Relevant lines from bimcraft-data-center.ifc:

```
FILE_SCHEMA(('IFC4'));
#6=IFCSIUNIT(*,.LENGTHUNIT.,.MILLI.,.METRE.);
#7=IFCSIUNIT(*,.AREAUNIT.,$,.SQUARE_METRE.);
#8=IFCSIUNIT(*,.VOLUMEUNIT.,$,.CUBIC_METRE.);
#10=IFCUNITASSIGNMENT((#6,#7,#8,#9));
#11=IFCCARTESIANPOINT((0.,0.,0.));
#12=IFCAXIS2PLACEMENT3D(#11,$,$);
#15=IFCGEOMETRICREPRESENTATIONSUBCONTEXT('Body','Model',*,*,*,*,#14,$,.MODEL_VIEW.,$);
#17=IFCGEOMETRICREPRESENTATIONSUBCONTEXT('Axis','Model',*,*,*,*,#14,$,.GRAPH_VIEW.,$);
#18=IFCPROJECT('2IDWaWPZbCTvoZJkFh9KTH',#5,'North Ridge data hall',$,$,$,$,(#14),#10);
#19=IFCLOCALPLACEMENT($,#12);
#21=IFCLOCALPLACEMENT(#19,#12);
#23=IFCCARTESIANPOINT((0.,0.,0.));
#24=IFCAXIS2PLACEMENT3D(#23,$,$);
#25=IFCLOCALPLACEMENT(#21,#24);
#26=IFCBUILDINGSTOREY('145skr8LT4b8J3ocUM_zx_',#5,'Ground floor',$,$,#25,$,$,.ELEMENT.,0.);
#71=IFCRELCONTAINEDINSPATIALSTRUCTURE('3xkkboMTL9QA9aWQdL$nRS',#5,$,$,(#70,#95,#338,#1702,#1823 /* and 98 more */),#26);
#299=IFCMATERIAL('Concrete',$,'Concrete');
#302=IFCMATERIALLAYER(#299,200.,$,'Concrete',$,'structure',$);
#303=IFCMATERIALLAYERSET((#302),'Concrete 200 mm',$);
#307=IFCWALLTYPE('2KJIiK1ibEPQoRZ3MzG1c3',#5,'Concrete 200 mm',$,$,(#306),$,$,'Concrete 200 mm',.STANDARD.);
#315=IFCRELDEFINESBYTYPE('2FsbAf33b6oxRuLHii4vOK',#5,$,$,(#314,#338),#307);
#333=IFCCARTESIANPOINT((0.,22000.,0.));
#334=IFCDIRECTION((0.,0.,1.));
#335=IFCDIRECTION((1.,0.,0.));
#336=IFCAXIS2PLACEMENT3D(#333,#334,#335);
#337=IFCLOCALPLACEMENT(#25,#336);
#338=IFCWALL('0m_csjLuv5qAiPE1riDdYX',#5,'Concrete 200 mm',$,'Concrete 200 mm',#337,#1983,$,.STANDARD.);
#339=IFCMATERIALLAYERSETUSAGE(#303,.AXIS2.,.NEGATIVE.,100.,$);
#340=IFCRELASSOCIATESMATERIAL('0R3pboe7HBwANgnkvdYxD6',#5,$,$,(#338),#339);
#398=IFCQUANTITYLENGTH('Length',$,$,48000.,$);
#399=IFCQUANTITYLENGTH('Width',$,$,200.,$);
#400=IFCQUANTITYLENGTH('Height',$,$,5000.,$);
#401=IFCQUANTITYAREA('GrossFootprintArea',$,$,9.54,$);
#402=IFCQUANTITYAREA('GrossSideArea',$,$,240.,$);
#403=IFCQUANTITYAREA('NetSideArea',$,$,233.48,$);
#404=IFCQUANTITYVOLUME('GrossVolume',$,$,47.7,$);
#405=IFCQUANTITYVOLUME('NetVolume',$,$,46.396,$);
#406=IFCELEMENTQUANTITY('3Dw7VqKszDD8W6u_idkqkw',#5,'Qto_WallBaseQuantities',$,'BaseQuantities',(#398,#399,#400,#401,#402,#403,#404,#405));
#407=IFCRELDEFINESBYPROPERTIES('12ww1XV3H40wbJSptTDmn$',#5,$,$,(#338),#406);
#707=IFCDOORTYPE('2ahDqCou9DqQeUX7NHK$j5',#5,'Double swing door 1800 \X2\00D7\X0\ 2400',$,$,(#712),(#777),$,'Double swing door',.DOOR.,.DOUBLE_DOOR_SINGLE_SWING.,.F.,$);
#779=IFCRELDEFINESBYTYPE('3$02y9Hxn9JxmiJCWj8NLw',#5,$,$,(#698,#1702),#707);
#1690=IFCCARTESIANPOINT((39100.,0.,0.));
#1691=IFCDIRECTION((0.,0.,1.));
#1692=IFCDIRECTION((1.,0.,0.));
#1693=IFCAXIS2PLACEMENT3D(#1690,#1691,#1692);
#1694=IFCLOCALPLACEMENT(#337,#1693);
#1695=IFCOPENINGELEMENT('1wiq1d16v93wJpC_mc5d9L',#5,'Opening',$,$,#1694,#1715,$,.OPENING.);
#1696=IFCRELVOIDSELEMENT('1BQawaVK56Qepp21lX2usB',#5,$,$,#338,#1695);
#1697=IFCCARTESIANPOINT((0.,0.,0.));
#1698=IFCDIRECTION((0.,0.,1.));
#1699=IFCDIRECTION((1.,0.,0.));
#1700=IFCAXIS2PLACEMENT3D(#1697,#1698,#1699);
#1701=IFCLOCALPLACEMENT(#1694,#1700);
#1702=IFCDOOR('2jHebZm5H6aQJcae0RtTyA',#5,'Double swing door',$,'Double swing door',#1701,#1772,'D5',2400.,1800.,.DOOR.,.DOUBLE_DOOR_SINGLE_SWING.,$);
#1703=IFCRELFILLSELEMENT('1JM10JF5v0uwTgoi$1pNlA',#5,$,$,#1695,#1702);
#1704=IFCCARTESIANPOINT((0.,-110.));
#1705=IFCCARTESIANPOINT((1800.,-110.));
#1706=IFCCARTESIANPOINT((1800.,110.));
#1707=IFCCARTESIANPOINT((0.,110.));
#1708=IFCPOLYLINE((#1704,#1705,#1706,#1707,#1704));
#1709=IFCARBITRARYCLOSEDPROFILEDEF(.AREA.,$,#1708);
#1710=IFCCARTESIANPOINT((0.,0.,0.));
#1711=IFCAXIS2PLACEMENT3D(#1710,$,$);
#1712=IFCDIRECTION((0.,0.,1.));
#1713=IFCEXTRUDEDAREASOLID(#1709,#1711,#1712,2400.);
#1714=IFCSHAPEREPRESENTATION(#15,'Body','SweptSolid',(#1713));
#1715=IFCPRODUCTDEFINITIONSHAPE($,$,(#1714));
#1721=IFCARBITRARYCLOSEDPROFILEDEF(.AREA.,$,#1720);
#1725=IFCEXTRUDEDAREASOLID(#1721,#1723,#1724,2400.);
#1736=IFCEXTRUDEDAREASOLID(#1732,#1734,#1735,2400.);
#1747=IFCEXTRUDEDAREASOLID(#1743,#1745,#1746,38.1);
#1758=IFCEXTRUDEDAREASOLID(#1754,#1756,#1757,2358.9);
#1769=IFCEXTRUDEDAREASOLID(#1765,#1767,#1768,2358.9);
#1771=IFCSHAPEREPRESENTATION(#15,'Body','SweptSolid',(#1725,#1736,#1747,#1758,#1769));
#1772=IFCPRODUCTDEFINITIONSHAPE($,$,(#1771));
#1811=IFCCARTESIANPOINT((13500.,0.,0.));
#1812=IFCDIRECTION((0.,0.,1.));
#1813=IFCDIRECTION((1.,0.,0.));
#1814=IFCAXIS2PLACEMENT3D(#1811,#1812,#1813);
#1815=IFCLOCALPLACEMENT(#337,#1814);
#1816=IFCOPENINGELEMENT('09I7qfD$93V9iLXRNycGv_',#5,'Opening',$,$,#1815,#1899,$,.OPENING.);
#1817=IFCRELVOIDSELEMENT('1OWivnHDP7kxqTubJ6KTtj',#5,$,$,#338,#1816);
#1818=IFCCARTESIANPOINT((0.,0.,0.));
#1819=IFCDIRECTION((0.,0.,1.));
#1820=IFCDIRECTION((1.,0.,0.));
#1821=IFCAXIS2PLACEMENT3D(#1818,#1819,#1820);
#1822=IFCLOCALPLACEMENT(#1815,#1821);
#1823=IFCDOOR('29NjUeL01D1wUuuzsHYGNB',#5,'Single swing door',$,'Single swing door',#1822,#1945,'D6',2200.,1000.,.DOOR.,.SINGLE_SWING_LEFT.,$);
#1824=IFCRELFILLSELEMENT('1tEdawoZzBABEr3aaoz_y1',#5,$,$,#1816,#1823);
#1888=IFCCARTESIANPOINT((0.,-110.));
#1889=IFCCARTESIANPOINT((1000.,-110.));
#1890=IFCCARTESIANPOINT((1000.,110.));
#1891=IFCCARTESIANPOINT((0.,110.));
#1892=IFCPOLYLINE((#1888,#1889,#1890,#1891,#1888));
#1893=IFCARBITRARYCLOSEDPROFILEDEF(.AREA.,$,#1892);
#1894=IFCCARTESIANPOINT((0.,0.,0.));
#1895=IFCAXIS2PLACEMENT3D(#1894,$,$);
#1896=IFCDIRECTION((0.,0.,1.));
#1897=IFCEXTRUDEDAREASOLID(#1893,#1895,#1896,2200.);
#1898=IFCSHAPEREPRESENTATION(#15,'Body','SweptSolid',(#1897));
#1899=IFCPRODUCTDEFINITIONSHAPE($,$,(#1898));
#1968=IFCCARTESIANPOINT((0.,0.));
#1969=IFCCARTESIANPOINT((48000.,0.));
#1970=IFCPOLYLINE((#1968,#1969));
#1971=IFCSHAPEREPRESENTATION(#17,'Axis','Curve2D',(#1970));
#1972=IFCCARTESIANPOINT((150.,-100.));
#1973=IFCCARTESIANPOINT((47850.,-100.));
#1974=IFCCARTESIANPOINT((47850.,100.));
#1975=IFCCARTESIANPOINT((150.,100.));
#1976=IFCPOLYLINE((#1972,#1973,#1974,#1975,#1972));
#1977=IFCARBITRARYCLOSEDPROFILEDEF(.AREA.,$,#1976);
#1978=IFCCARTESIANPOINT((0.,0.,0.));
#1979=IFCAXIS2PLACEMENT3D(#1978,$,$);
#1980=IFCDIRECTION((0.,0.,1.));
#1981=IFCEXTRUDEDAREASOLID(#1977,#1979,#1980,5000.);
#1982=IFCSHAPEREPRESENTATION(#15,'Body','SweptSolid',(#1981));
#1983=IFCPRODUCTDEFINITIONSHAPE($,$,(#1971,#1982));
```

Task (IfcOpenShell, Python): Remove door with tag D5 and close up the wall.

```python
import ifcopenshell
import ifcopenshell.api.feature
import ifcopenshell.api.pset
import ifcopenshell.api.root
import ifcopenshell.geom
import ifcopenshell.util.element
import ifcopenshell.util.shape
import ifcopenshell.util.unit

model = ifcopenshell.open("bimcraft-data-center.ifc")
area_scale = ifcopenshell.util.unit.calculate_unit_scale(model, "AREAUNIT")
volume_scale = ifcopenshell.util.unit.calculate_unit_scale(model, "VOLUMEUNIT")
settings = ifcopenshell.geom.settings()


def volume(element):
    """Net volume in cubic metres, openings subtracted."""
    shape = ifcopenshell.geom.create_shape(settings, element)
    return ifcopenshell.util.shape.get_volume(shape.geometry)


door = model.by_id(1702)
opening = door.FillsVoids[0].RelatingOpeningElement
wall = opening.VoidsElements[0].RelatingBuildingElement
before = volume(wall)

ifcopenshell.api.root.remove_product(model, product=door)
ifcopenshell.api.feature.remove_feature(model, feature=opening)

after = volume(wall)
thickness = 0.2  # wall thickness in metres

# Update the wall's stored quantities.
qto = model.by_id(ifcopenshell.util.element.get_pset(wall, "Qto_WallBaseQuantities", should_inherit=False)["id"])
ifcopenshell.api.pset.edit_qto(model, qto=qto, properties={
    "NetSideArea": after / thickness / area_scale,
    "NetVolume": after / volume_scale,
})

print(f"wall volume {before:.3f} -> {after:.3f} m3")

model.write("bimcraft-data-center_edited.ifc")
```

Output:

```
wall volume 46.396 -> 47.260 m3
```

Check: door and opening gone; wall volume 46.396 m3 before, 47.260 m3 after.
